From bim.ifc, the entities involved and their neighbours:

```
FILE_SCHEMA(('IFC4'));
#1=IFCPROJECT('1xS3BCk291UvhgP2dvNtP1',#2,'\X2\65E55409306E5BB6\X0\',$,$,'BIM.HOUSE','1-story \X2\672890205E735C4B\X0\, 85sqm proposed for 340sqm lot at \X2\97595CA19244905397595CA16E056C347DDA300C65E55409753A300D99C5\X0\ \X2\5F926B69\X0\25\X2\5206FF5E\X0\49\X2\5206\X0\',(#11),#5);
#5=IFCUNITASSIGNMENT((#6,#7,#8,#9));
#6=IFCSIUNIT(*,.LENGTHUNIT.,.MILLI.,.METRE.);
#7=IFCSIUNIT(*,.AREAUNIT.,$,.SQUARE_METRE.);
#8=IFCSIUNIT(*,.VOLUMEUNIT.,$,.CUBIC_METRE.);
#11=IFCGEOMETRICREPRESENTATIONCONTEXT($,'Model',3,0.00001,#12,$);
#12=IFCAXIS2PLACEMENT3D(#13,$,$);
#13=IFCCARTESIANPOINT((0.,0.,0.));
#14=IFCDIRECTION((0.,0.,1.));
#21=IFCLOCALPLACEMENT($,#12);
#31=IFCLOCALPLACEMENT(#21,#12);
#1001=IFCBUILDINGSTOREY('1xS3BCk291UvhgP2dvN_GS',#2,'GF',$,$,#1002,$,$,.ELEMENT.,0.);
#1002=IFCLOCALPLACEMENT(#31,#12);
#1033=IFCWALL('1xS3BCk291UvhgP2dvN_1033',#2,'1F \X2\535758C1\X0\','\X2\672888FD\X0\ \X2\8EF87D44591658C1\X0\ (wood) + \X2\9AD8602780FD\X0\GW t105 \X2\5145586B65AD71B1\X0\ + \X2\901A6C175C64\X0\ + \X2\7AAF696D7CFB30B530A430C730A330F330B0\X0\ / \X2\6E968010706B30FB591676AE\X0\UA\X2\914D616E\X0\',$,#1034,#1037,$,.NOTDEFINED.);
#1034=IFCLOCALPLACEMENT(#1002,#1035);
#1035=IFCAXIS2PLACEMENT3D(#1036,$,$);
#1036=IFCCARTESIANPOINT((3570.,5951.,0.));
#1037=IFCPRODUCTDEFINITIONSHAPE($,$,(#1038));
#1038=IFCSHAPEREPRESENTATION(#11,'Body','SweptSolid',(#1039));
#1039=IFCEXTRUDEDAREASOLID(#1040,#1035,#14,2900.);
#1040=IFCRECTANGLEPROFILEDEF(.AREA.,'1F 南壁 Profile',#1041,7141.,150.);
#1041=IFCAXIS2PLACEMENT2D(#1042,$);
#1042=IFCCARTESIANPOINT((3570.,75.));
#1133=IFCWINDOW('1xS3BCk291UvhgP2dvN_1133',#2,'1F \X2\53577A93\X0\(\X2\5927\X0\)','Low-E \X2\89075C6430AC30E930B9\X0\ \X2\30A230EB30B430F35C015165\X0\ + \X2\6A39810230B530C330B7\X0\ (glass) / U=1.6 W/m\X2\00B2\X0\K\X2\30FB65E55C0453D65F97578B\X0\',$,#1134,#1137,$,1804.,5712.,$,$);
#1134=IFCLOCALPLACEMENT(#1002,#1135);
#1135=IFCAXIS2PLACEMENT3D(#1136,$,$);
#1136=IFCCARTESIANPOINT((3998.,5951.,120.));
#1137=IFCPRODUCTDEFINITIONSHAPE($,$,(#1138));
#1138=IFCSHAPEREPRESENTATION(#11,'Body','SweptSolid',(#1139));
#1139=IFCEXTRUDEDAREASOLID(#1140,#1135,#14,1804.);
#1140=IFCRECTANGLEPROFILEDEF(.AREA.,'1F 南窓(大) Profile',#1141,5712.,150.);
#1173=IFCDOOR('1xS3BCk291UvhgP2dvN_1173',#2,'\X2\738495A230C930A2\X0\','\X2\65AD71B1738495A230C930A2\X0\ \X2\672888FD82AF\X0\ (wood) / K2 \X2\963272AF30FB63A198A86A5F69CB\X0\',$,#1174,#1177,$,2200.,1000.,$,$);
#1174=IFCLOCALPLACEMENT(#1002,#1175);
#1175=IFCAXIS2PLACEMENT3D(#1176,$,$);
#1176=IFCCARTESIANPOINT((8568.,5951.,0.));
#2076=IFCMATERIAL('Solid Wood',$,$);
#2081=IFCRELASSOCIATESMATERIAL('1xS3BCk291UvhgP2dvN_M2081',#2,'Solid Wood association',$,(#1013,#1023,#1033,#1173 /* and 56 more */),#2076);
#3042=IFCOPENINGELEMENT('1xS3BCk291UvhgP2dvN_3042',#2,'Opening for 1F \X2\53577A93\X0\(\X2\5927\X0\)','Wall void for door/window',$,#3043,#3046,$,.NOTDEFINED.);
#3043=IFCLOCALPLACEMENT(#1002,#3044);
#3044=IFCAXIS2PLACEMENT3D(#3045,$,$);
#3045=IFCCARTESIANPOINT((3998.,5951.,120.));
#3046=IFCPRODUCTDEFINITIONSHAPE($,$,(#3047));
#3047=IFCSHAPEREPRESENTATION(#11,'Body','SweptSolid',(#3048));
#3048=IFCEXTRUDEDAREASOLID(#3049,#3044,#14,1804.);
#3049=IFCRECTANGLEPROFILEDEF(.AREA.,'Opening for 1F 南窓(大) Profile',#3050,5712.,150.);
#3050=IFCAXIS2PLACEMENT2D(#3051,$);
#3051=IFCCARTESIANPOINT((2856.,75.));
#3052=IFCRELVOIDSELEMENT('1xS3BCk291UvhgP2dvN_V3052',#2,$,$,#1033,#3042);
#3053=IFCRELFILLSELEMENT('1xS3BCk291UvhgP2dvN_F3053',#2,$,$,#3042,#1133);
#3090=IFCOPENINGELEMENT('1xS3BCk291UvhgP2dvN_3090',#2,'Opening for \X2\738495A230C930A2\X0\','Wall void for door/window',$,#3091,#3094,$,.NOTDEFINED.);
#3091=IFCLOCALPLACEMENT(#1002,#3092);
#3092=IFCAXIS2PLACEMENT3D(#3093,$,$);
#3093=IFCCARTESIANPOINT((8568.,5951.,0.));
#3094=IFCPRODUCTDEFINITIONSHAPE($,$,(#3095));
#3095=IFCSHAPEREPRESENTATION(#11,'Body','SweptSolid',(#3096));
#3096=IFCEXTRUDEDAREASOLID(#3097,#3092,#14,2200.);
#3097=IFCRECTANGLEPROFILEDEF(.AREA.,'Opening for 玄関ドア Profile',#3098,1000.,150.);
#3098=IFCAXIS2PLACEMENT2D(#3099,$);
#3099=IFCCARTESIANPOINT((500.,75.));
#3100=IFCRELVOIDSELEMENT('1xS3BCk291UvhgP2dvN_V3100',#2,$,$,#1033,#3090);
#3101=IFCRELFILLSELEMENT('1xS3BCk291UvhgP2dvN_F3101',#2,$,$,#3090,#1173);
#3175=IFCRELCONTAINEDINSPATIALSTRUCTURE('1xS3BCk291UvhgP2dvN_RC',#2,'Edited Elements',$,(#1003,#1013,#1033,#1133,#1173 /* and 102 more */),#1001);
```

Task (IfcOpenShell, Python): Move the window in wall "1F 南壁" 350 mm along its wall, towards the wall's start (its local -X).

```python
import ifcopenshell
import ifcopenshell.api.geometry
import ifcopenshell.util.placement
import ifcopenshell.util.unit

model = ifcopenshell.open("bim.ifc")
unit_scale = ifcopenshell.util.unit.calculate_unit_scale(model)

window = model.by_guid("1xS3BCk291UvhgP2dvN_1133")
opening = window.FillsVoids[0].RelatingOpeningElement
wall = opening.VoidsElements[0].RelatingBuildingElement

wall_matrix = ifcopenshell.util.placement.get_local_placement(wall.ObjectPlacement)
shift = wall_matrix[:3, 0] * -0.35 / unit_scale
before = ifcopenshell.util.placement.get_local_placement(window.ObjectPlacement)[:3, 3].copy()

# The window is not placed relative to its opening, so move both.
for product in (opening, window):
    matrix = ifcopenshell.util.placement.get_local_placement(product.ObjectPlacement)
    matrix[:3, 3] += shift
    ifcopenshell.api.geometry.edit_object_placement(model, product=product, matrix=matrix, is_si=False)

after = ifcopenshell.util.placement.get_local_placement(window.ObjectPlacement)[:3, 3]
print("window moved by", (after - before).round(3) + 0.0)

model.write("bim_rev.ifc")
```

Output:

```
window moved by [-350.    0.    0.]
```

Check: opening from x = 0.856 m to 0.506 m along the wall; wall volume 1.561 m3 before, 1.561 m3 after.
